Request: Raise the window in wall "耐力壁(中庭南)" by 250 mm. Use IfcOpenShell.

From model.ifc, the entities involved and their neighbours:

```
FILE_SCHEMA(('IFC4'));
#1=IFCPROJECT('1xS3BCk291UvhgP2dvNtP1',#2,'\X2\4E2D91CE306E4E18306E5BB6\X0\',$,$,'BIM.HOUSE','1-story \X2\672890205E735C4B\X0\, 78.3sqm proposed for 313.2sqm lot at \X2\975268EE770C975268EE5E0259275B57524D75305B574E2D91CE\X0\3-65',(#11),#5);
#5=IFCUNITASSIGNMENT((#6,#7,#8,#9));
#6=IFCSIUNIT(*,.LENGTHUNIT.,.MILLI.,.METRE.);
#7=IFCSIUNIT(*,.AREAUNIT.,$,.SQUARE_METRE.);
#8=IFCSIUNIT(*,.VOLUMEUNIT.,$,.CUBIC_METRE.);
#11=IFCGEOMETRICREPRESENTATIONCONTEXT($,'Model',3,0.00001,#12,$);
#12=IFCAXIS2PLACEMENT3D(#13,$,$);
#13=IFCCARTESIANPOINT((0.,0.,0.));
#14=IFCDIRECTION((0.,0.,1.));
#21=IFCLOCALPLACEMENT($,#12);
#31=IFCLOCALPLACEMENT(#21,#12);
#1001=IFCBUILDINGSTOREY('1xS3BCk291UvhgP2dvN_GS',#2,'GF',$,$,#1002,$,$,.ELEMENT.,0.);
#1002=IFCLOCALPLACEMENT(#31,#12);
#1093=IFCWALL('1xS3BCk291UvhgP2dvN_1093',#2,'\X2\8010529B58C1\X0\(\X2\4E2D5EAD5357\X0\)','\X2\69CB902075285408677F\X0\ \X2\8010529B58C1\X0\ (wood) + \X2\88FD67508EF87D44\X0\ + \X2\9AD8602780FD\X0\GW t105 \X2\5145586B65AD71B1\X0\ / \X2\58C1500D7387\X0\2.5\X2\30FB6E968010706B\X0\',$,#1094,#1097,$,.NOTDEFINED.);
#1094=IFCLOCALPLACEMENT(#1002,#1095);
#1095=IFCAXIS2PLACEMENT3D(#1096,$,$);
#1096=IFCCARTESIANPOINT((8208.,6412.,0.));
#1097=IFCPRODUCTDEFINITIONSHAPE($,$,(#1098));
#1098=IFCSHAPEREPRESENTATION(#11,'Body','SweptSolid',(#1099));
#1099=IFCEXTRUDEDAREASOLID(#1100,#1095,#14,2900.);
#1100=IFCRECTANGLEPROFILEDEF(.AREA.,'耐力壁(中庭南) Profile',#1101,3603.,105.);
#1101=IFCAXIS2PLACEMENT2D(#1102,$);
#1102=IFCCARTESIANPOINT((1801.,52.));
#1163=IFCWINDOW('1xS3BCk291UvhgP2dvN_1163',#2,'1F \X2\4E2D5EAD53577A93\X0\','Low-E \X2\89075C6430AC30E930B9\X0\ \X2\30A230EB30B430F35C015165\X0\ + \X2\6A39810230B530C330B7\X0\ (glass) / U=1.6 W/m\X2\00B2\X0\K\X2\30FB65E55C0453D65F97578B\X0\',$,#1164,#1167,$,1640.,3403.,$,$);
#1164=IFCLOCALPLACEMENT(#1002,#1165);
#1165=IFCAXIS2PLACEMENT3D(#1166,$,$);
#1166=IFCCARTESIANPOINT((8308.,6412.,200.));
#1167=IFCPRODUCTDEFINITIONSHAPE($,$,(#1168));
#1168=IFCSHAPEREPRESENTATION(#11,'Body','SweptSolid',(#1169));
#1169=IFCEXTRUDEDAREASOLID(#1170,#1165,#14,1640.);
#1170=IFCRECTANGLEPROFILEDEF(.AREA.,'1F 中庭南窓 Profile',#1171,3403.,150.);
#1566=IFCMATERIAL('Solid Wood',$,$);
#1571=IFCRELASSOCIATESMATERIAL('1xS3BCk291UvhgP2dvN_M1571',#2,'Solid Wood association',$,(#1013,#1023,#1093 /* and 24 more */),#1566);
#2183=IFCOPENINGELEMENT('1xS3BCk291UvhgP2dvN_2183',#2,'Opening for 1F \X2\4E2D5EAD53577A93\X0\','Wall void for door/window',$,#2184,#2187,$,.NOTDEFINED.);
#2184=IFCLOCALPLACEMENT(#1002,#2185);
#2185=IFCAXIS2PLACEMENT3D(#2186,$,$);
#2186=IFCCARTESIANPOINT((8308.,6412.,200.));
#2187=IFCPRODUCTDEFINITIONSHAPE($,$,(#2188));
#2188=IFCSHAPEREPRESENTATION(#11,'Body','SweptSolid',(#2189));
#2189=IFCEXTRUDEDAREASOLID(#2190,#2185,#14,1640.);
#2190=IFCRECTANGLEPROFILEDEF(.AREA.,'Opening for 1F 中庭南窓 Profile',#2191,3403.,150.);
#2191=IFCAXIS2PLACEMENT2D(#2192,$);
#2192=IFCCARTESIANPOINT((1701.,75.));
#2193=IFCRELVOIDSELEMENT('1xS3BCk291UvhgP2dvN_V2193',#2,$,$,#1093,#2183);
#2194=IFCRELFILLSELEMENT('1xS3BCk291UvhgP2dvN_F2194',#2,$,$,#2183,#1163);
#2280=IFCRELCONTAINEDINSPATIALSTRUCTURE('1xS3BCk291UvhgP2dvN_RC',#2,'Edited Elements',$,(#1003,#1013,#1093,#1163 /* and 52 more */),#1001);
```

```python
import numpy as np
import ifcopenshell
import ifcopenshell.api.geometry
import ifcopenshell.util.placement
import ifcopenshell.util.unit

model = ifcopenshell.open("model.ifc")
unit_scale = ifcopenshell.util.unit.calculate_unit_scale(model)

window = model.by_guid("1xS3BCk291UvhgP2dvN_1163")
opening = window.FillsVoids[0].RelatingOpeningElement
dz = 0.25 / unit_scale

shift = np.array([0.0, 0.0, dz])
# The window is not placed relative to its opening, so move both.
for product in (opening, window):
    matrix = ifcopenshell.util.placement.get_local_placement(product.ObjectPlacement)
    matrix[:3, 3] += shift
    ifcopenshell.api.geometry.edit_object_placement(model, product=product, matrix=matrix, is_si=False)

print(f"moved by {dz * unit_scale:+.3f} m")

model.write("model_updated.ifc")
```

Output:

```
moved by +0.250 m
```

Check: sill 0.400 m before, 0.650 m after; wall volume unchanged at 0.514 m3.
